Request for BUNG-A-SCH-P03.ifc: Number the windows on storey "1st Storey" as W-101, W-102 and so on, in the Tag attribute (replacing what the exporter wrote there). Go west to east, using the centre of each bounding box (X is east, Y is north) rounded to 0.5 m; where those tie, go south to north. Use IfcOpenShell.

First a look at what the model holds.

```python
import ifcopenshell
import ifcopenshell.util.element
import ifcopenshell.util.placement

model = ifcopenshell.open("BUNG-A-SCH-P03.ifc")
print(model.schema)
storey = next(s for s in model.by_type("IfcBuildingStorey") if s.Name == "1st Storey")
windows = [e for e in ifcopenshell.util.element.get_decomposition(storey) if e.is_a("IfcWindow")]
for e in sorted(windows, key=lambda e: e.id()):
    origin = ifcopenshell.util.placement.get_local_placement(e.ObjectPlacement)[:3, 3]
    print(e.id(), e.Tag, e.Name, origin.round(2) + 0.0, sep=" | ")
```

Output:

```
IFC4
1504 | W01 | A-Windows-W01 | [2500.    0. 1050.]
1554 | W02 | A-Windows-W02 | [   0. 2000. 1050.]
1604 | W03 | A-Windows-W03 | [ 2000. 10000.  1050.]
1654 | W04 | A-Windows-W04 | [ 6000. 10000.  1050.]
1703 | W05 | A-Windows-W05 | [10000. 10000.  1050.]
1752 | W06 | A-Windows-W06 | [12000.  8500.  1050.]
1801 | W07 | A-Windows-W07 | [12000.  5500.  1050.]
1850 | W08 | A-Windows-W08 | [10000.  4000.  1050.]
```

```python
import ifcopenshell
import ifcopenshell.geom
import ifcopenshell.util.element
import ifcopenshell.util.shape

model = ifcopenshell.open("BUNG-A-SCH-P03.ifc")
settings = ifcopenshell.geom.settings()
settings.set("use-world-coords", True)


def centre(element):
    shape = ifcopenshell.geom.create_shape(settings, element)
    return ifcopenshell.util.shape.get_bbox_centroid(shape.geometry)


storey = next(s for s in model.by_type("IfcBuildingStorey") if s.Name == "1st Storey")
windows = [e for e in ifcopenshell.util.element.get_decomposition(storey) if e.is_a("IfcWindow")]

# Insertion points can sit at a corner or the storey origin, so sort by the geometry (in metres).
centres = {e: centre(e) for e in windows}
windows.sort(key=lambda e: (round(centres[e][0] / 0.5), centres[e][1]))

for i, e in enumerate(windows, start=1):
    number = f"W-1{i:02d}"
    e.Tag = number
    print(e.id(), number)

model.write("BUNG-A-SCH-P03_rev.ifc")
```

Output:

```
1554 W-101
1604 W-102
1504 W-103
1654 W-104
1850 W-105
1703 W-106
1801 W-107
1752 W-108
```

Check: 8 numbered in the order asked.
